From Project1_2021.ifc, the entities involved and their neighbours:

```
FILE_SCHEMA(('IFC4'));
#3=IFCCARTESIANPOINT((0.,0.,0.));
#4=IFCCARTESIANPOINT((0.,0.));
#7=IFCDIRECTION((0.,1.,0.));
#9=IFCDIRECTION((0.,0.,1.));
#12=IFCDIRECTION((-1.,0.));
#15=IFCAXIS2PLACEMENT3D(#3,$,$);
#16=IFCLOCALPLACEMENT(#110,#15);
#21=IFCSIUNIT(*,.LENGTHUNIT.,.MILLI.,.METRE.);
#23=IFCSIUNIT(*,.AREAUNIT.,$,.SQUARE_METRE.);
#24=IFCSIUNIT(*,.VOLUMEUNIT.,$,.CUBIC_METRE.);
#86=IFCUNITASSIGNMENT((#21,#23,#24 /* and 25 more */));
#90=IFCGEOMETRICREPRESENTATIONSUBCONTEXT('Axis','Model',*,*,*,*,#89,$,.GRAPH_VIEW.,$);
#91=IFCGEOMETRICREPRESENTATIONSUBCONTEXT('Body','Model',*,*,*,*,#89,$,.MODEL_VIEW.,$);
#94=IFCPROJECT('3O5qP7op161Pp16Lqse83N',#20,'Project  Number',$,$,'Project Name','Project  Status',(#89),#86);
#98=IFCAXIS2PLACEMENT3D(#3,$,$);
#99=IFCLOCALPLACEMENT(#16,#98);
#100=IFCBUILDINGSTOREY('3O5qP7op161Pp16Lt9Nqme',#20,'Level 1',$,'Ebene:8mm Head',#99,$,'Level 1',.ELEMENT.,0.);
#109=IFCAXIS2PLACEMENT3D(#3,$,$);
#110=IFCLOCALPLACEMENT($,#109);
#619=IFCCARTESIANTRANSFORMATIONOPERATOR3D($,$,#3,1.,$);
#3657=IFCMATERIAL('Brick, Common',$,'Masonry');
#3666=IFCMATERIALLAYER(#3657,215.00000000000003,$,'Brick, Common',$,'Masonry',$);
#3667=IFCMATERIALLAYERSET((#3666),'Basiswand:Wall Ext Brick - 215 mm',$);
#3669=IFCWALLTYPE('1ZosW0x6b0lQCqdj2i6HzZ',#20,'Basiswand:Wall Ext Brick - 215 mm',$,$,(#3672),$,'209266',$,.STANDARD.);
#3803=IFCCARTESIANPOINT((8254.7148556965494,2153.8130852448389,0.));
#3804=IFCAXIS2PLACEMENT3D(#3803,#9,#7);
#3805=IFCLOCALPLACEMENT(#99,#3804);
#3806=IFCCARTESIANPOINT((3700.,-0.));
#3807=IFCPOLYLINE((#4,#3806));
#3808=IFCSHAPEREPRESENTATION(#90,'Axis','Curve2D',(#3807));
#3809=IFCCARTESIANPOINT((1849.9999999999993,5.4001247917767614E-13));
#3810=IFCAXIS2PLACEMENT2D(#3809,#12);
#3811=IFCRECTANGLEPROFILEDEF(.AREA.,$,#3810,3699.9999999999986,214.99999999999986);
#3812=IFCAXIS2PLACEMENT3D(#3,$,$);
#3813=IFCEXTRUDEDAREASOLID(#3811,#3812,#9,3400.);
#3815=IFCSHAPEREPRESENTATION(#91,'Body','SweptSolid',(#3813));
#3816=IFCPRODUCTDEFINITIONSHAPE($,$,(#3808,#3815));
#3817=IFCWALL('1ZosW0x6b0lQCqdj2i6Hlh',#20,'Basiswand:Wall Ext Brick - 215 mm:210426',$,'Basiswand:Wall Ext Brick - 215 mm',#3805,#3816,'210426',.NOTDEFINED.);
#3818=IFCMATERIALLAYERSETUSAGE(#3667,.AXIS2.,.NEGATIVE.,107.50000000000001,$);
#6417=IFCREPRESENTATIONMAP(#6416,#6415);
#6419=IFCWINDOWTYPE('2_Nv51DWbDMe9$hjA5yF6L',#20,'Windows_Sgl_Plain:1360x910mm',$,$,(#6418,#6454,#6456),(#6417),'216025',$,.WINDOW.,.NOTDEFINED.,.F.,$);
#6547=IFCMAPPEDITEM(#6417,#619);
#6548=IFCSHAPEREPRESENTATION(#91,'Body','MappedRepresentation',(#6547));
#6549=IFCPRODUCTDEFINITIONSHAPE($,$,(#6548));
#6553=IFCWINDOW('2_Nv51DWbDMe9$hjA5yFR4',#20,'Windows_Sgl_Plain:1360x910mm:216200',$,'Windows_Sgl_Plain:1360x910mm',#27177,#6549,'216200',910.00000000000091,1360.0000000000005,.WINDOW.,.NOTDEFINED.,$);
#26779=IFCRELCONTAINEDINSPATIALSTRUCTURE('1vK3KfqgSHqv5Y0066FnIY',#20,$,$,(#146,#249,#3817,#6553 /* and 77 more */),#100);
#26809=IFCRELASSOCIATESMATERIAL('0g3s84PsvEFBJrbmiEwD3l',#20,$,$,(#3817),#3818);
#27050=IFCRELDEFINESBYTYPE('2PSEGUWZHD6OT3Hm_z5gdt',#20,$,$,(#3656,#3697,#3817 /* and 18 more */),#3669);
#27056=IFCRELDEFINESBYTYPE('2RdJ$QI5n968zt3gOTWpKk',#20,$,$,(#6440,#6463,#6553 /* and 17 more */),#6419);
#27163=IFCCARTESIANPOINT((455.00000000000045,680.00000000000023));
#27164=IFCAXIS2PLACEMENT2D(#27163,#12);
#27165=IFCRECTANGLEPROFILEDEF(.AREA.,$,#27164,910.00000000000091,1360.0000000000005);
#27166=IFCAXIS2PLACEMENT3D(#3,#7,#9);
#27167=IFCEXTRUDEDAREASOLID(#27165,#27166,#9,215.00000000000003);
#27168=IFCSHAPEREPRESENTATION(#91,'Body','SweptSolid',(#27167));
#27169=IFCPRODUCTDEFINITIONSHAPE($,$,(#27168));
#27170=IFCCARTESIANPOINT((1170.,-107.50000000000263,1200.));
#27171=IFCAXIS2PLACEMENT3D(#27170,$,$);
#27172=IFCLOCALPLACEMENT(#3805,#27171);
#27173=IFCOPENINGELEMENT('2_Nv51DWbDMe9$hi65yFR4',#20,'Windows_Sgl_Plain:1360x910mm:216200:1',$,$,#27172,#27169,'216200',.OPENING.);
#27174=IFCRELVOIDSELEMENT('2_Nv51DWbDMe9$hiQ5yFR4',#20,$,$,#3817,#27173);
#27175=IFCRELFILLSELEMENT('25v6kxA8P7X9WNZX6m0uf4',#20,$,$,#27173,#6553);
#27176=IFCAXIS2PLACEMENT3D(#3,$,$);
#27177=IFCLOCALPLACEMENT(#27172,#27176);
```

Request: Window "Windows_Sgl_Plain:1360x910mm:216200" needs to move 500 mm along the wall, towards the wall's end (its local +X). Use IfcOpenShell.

```python
import ifcopenshell
import ifcopenshell.api.geometry
import ifcopenshell.util.placement

model = ifcopenshell.open("Project1_2021.ifc")

window = model.by_guid("2_Nv51DWbDMe9$hjA5yFR4")
opening = window.FillsVoids[0].RelatingOpeningElement
wall = opening.VoidsElements[0].RelatingBuildingElement

wall_matrix = ifcopenshell.util.placement.get_local_placement(wall.ObjectPlacement)
shift = wall_matrix[:3, 0] * 500.0
before = ifcopenshell.util.placement.get_local_placement(window.ObjectPlacement)[:3, 3].copy()

# The window is placed relative to its opening, so it follows when the opening moves.
matrix = ifcopenshell.util.placement.get_local_placement(opening.ObjectPlacement)
matrix[:3, 3] += shift
ifcopenshell.api.geometry.edit_object_placement(
    model, product=opening, matrix=matrix, is_si=False, should_transform_children=True
)

after = ifcopenshell.util.placement.get_local_placement(window.ObjectPlacement)[:3, 3]
print("window moved by", (after - before).round(3) + 0.0)

model.write("Project1_2021_edited.ifc")
```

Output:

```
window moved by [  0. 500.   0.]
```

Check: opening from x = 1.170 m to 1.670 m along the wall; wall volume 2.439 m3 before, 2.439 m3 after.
